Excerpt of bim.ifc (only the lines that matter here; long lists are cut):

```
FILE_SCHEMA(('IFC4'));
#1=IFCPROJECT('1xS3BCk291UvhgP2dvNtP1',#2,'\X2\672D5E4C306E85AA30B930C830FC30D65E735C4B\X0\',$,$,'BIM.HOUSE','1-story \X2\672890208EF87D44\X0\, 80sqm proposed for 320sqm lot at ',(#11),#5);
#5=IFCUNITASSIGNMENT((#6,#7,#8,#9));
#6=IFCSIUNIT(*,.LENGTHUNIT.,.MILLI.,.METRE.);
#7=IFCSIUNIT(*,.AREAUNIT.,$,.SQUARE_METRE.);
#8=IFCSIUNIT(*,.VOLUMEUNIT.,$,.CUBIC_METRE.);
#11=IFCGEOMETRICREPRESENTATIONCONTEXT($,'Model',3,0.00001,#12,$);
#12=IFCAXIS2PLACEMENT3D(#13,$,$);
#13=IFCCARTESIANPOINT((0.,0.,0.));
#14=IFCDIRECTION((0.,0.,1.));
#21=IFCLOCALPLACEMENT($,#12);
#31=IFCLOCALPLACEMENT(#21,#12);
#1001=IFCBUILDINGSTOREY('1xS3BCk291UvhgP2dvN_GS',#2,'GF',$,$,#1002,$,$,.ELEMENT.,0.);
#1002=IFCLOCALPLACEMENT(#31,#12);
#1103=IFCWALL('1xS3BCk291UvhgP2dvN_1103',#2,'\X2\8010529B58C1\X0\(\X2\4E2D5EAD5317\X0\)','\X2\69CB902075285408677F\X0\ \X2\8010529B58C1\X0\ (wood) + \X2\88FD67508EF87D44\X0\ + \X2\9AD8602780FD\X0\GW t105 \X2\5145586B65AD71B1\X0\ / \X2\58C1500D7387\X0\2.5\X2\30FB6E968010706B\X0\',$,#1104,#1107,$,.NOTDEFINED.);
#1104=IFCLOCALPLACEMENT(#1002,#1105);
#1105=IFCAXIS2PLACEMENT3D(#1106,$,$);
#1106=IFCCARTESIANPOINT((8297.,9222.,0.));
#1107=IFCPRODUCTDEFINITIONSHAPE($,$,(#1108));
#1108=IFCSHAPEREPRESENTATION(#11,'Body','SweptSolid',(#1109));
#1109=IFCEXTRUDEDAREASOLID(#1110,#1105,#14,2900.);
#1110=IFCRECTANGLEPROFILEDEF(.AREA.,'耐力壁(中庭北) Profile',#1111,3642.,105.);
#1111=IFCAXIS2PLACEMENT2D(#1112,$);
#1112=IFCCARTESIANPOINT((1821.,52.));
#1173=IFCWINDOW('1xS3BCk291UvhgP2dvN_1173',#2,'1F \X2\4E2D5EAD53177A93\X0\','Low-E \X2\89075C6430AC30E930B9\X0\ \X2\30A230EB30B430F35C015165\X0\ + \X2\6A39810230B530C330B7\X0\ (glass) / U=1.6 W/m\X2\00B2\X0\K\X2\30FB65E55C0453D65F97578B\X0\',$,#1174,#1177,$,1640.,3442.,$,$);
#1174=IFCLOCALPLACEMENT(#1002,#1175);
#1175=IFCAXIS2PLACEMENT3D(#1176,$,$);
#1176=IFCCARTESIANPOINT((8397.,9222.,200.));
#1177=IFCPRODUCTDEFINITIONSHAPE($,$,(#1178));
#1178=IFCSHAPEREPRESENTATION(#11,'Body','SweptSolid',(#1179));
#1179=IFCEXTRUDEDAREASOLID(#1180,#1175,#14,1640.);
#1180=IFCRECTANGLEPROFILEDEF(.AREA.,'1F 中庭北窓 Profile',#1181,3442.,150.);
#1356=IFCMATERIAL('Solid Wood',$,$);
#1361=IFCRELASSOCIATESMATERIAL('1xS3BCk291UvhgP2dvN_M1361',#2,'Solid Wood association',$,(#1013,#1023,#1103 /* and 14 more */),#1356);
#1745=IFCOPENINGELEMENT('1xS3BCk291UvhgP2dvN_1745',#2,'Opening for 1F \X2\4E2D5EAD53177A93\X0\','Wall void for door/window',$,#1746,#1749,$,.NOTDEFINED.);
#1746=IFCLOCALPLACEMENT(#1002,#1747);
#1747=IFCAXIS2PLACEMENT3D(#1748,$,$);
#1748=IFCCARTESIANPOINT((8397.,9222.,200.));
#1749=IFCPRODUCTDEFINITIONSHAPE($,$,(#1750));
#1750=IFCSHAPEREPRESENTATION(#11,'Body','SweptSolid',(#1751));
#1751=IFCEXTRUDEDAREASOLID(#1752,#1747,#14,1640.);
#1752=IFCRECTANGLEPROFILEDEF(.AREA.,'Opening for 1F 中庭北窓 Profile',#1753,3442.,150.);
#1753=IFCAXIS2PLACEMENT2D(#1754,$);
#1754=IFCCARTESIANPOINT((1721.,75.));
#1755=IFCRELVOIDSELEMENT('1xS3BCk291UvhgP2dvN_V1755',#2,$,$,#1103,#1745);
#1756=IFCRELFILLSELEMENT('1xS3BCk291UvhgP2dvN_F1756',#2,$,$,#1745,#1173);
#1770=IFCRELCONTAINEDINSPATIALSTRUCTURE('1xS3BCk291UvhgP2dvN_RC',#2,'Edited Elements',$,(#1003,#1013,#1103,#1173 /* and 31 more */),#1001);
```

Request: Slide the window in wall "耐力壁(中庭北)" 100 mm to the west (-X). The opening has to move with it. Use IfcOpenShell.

```python
import ifcopenshell
import ifcopenshell.api.geometry
import ifcopenshell.util.placement
import ifcopenshell.util.unit

model = ifcopenshell.open("bim.ifc")
unit_scale = ifcopenshell.util.unit.calculate_unit_scale(model)

window = model.by_guid("1xS3BCk291UvhgP2dvN_1173")
opening = window.FillsVoids[0].RelatingOpeningElement
wall = opening.VoidsElements[0].RelatingBuildingElement

wall_matrix = ifcopenshell.util.placement.get_local_placement(wall.ObjectPlacement)
shift = wall_matrix[:3, 0] * -0.1 / unit_scale
before = ifcopenshell.util.placement.get_local_placement(window.ObjectPlacement)[:3, 3].copy()

# The window is not placed relative to its opening, so move both.
for product in (opening, window):
    matrix = ifcopenshell.util.placement.get_local_placement(product.ObjectPlacement)
    matrix[:3, 3] += shift
    ifcopenshell.api.geometry.edit_object_placement(model, product=product, matrix=matrix, is_si=False)

after = ifcopenshell.util.placement.get_local_placement(window.ObjectPlacement)[:3, 3]
print("window moved by", (after - before).round(3) + 0.0)

model.write("bim_v2.ifc")
```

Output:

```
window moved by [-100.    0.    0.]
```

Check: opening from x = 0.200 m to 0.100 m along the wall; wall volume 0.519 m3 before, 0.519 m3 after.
